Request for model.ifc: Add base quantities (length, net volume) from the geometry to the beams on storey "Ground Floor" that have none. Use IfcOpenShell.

First a look at what the model holds.

```python
import ifcopenshell
import ifcopenshell.util.element
import ifcopenshell.util.unit

model = ifcopenshell.open("model.ifc")
print(model.schema)
for unit_type in ("LENGTHUNIT", "AREAUNIT", "VOLUMEUNIT"):
    print(unit_type, ifcopenshell.util.unit.calculate_unit_scale(model, unit_type))
storey = next(s for s in model.by_type("IfcBuildingStorey") if s.Name == "Ground Floor")
beams = [e for e in ifcopenshell.util.element.get_decomposition(storey) if e.is_a("IfcBeam")]
for e in sorted(beams, key=lambda e: e.id()):
    print(e.id(), e.is_a(), e.Name, list(ifcopenshell.util.element.get_psets(e, qtos_only=True)), sep=" | ")
```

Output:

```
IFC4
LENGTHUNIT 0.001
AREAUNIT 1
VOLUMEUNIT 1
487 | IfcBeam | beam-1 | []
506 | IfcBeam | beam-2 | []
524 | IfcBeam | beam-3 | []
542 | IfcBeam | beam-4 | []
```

```python
import ifcopenshell
import ifcopenshell.api.pset
import ifcopenshell.geom
import ifcopenshell.util.element
import ifcopenshell.util.shape
import ifcopenshell.util.unit

model = ifcopenshell.open("model.ifc")
unit_scale = ifcopenshell.util.unit.calculate_unit_scale(model)
volume_scale = ifcopenshell.util.unit.calculate_unit_scale(model, "VOLUMEUNIT")
settings = ifcopenshell.geom.settings()

storey = next(s for s in model.by_type("IfcBuildingStorey") if s.Name == "Ground Floor")
beams = [e for e in ifcopenshell.util.element.get_decomposition(storey) if e.is_a("IfcBeam")]

for e in sorted(beams, key=lambda e: e.id()):
    if ifcopenshell.util.element.get_psets(e, qtos_only=True, should_inherit=False):
        continue
    # Geometry comes back in metres, in the element's own axes.
    shape = ifcopenshell.geom.create_shape(settings, e)
    values = {
        "Length": ifcopenshell.util.shape.get_max_xyz(shape.geometry) / unit_scale,
        "NetVolume": ifcopenshell.util.shape.get_volume(shape.geometry) / volume_scale,
    }
    qto = ifcopenshell.api.pset.add_qto(model, product=e, name="Qto_BeamBaseQuantities")
    ifcopenshell.api.pset.edit_qto(model, qto=qto, properties=values)
    print(e.id(), {k: round(v, 3) for k, v in values.items()})

model.write("model_rev.ifc")
```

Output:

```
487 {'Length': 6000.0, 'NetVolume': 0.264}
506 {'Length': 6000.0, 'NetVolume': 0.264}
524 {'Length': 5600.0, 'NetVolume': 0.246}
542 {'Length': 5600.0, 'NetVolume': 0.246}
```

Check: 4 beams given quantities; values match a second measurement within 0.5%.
